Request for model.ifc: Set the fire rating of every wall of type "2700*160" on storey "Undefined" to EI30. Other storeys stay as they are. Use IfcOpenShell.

First a look at what the model holds.

```python
import ifcopenshell
import ifcopenshell.util.element

model = ifcopenshell.open("model.ifc")
print(model.schema)
storey = next(s for s in model.by_type("IfcBuildingStorey") if s.Name == "Undefined")
walls = [e for e in ifcopenshell.util.element.get_decomposition(storey) if e.is_a("IfcWall")]
seen = {}
for e in walls:
    element_type = ifcopenshell.util.element.get_type(e)
    key = (element_type.Name if element_type != e and element_type else None, ifcopenshell.util.element.get_pset(e, "Pset_WallCommon", "FireRating"))
    seen[key] = seen.get(key, 0) + 1
for (name, value), count in sorted(seen.items(), key=str):
    print(count, "x", name, "|", value)
```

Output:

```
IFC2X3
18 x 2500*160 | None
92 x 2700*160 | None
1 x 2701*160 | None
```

```python
import ifcopenshell
import ifcopenshell.api.pset
import ifcopenshell.util.element

model = ifcopenshell.open("model.ifc")

storey = next(s for s in model.by_type("IfcBuildingStorey") if s.Name == "Undefined")
walls = [e for e in ifcopenshell.util.element.get_decomposition(storey) if e.is_a("IfcWall")]

count = 0
for e in walls:
    element_type = ifcopenshell.util.element.get_type(e)
    if element_type in (None, e) or element_type.Name != "2700*160":
        continue
    # add_pset returns the element's existing set when there is one.
    pset = ifcopenshell.api.pset.add_pset(model, product=e, name="Pset_WallCommon")
    ifcopenshell.api.pset.edit_pset(model, pset=pset, properties={"FireRating": "EI30"})
    count += 1

print(count, "walls updated")

model.write("model_rev.ifc")
```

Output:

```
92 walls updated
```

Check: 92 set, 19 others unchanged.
